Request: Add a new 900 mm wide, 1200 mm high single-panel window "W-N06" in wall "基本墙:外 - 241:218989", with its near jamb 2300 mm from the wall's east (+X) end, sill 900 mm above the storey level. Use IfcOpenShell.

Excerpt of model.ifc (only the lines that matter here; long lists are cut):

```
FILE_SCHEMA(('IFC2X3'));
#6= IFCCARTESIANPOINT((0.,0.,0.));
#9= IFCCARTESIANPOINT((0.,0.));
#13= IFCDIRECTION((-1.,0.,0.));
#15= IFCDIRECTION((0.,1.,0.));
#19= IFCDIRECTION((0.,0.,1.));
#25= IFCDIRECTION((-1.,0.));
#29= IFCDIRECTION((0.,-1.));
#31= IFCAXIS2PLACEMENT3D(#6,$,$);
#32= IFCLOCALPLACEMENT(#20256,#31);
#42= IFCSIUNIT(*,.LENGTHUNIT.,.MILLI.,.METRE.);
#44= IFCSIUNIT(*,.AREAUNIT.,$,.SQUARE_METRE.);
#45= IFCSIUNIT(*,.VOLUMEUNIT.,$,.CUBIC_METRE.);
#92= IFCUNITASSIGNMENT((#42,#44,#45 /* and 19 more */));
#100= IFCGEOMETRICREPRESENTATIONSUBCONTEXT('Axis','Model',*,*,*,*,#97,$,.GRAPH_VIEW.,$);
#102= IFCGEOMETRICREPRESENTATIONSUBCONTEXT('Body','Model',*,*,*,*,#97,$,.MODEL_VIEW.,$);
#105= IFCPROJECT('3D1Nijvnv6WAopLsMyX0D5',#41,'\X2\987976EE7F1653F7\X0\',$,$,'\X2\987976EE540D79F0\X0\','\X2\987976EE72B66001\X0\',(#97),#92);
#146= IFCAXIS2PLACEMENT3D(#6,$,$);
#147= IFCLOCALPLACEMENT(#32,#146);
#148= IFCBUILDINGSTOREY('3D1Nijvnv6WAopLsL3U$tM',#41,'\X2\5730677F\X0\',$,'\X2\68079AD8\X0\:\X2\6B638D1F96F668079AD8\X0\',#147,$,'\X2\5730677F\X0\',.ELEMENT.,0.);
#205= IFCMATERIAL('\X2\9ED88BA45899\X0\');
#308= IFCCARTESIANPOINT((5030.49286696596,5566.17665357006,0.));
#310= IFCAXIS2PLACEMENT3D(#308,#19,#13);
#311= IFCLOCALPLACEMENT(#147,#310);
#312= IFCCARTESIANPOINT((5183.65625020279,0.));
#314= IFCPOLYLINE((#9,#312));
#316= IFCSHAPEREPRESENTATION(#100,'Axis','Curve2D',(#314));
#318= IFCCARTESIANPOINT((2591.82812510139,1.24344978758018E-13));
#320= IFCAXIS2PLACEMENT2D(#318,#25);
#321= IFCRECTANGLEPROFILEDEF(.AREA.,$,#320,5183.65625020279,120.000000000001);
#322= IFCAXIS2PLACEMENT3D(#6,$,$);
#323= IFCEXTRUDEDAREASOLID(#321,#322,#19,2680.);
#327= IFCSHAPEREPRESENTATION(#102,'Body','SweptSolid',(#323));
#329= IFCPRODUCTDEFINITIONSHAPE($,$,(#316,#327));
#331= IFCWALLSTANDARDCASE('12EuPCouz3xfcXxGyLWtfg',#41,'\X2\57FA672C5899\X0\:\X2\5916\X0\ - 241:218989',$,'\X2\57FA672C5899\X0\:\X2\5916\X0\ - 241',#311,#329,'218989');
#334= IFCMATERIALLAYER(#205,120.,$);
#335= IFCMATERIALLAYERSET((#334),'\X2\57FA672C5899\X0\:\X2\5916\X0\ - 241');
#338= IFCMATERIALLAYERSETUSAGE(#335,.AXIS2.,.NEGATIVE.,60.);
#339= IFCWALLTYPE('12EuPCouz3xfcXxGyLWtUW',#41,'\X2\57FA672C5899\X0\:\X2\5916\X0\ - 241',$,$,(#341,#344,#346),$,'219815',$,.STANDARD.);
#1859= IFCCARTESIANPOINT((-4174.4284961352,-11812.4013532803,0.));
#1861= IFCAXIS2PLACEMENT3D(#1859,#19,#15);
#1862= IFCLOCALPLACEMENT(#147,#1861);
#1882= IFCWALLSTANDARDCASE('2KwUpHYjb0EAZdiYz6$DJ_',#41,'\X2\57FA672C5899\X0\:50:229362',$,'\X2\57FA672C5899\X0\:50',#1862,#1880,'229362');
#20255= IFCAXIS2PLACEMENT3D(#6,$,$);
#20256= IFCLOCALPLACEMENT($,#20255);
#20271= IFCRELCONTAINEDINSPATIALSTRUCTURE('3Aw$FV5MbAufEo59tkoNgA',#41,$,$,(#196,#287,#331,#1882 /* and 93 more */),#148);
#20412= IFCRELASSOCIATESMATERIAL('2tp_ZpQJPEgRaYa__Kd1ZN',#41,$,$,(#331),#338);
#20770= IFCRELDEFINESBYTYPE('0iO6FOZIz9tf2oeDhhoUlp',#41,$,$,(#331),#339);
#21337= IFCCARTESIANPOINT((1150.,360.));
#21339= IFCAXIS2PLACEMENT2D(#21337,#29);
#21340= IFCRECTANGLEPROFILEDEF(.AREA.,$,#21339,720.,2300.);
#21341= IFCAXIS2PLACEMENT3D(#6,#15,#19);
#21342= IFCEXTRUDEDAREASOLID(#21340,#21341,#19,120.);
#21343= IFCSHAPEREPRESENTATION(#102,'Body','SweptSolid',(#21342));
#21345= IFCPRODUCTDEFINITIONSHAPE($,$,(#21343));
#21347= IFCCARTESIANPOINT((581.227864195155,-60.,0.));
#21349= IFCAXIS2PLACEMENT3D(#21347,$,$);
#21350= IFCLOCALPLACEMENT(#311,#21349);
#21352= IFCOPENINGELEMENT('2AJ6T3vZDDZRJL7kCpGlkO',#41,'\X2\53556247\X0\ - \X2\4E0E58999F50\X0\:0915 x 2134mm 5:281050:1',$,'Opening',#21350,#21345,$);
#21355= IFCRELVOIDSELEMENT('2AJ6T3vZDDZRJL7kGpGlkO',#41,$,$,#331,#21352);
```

```python
import numpy as np
import ifcopenshell
import ifcopenshell.api.feature
import ifcopenshell.api.geometry
import ifcopenshell.api.root
import ifcopenshell.api.spatial
import ifcopenshell.api.type
import ifcopenshell.geom
import ifcopenshell.util.element
import ifcopenshell.util.placement
import ifcopenshell.util.representation
import ifcopenshell.util.shape
import ifcopenshell.util.unit

model = ifcopenshell.open("model.ifc")
unit_scale = ifcopenshell.util.unit.calculate_unit_scale(model)
settings = ifcopenshell.geom.settings()


def volume(element):
    """Net volume in cubic metres, openings subtracted."""
    shape = ifcopenshell.geom.create_shape(settings, element)
    return ifcopenshell.util.shape.get_volume(shape.geometry)


wall = model.by_guid("12EuPCouz3xfcXxGyLWtfg")
storey = ifcopenshell.util.element.get_container(wall, ifc_class="IfcBuildingStorey")
context = ifcopenshell.util.representation.get_context(model, "Model", "Body", "MODEL_VIEW")
before = volume(wall)

width, height, from_end, sill = 0.9, 1.2, 2.3, 0.9  # metres

# The wall runs along its own X axis, and the end named is its -X end.
wall_shape = ifcopenshell.geom.create_shape(settings, wall)
x, y, z = ifcopenshell.util.shape.get_vertices(wall_shape.geometry).T
start = x.min() + from_end
face, thickness = float(y.min()), float(y.max() - y.min())
wall_matrix = ifcopenshell.util.placement.get_local_placement(wall.ObjectPlacement)
level = ifcopenshell.util.placement.get_local_placement(storey.ObjectPlacement)[2, 3]


def in_wall(x, y):
    """Placement at x, y metres in the wall's axes, at sill height."""
    matrix = wall_matrix.copy()
    matrix[:, 3] = wall_matrix @ np.array([x / unit_scale, y / unit_scale, 0.0, 1.0])
    matrix[2, 3] = level + sill / unit_scale
    return matrix


# Opening: a box that overshoots both wall faces by 50 mm.
opening = ifcopenshell.api.root.create_entity(model, ifc_class="IfcOpeningElement")
box = ifcopenshell.api.geometry.add_wall_representation(
    model, context=context, length=width, height=height, thickness=thickness + 0.1
)
ifcopenshell.api.geometry.assign_representation(model, product=opening, representation=box)
ifcopenshell.api.geometry.edit_object_placement(model, product=opening, matrix=in_wall(start, face - 0.05), is_si=False)
ifcopenshell.api.feature.add_feature(model, feature=opening, element=wall)

window = ifcopenshell.api.root.create_entity(model, ifc_class="IfcWindow", name="W-N06")
window.OverallWidth, window.OverallHeight = width / unit_scale, height / unit_scale
body = ifcopenshell.api.geometry.add_window_representation(
    model,
    context=context,
    overall_width=window.OverallWidth,
    overall_height=window.OverallHeight,
    partition_type="SINGLE_PANEL",
)
ifcopenshell.api.geometry.assign_representation(model, product=window, representation=body)
ifcopenshell.api.spatial.assign_container(model, products=[window], relating_structure=storey)
fills = ifcopenshell.api.feature.add_filling(model, opening=opening, element=window)
fills.OwnerHistory = window.OwnerHistory  # required in IFC2X3

# IFC2X3 keeps the operation on the window style.
style = ifcopenshell.api.root.create_entity(model, ifc_class="IfcWindowStyle", name="W-N06")
style.OperationType, style.ConstructionType = "SINGLE_PANEL", "NOTDEFINED"
style.ParameterTakesPrecedence = style.Sizeable = False
ifcopenshell.api.type.assign_type(model, related_objects=[window], relating_type=style)

# Centre the window in the wall's thickness.
ifcopenshell.api.geometry.edit_object_placement(model, product=window, matrix=in_wall(start, face), is_si=False)
window_shape = ifcopenshell.geom.create_shape(settings, window)
depth = ifcopenshell.util.shape.get_vertices(window_shape.geometry)[:, 1]
offset = face + thickness / 2 - (depth.min() + depth.max()) / 2
ifcopenshell.api.geometry.edit_object_placement(model, product=window, matrix=in_wall(start, offset), is_si=False)

after = volume(wall)

print(f"wall volume {before:.3f} -> {after:.3f} m3")

model.write("model-out.ifc")
```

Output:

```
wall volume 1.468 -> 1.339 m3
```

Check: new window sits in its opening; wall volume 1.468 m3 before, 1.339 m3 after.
